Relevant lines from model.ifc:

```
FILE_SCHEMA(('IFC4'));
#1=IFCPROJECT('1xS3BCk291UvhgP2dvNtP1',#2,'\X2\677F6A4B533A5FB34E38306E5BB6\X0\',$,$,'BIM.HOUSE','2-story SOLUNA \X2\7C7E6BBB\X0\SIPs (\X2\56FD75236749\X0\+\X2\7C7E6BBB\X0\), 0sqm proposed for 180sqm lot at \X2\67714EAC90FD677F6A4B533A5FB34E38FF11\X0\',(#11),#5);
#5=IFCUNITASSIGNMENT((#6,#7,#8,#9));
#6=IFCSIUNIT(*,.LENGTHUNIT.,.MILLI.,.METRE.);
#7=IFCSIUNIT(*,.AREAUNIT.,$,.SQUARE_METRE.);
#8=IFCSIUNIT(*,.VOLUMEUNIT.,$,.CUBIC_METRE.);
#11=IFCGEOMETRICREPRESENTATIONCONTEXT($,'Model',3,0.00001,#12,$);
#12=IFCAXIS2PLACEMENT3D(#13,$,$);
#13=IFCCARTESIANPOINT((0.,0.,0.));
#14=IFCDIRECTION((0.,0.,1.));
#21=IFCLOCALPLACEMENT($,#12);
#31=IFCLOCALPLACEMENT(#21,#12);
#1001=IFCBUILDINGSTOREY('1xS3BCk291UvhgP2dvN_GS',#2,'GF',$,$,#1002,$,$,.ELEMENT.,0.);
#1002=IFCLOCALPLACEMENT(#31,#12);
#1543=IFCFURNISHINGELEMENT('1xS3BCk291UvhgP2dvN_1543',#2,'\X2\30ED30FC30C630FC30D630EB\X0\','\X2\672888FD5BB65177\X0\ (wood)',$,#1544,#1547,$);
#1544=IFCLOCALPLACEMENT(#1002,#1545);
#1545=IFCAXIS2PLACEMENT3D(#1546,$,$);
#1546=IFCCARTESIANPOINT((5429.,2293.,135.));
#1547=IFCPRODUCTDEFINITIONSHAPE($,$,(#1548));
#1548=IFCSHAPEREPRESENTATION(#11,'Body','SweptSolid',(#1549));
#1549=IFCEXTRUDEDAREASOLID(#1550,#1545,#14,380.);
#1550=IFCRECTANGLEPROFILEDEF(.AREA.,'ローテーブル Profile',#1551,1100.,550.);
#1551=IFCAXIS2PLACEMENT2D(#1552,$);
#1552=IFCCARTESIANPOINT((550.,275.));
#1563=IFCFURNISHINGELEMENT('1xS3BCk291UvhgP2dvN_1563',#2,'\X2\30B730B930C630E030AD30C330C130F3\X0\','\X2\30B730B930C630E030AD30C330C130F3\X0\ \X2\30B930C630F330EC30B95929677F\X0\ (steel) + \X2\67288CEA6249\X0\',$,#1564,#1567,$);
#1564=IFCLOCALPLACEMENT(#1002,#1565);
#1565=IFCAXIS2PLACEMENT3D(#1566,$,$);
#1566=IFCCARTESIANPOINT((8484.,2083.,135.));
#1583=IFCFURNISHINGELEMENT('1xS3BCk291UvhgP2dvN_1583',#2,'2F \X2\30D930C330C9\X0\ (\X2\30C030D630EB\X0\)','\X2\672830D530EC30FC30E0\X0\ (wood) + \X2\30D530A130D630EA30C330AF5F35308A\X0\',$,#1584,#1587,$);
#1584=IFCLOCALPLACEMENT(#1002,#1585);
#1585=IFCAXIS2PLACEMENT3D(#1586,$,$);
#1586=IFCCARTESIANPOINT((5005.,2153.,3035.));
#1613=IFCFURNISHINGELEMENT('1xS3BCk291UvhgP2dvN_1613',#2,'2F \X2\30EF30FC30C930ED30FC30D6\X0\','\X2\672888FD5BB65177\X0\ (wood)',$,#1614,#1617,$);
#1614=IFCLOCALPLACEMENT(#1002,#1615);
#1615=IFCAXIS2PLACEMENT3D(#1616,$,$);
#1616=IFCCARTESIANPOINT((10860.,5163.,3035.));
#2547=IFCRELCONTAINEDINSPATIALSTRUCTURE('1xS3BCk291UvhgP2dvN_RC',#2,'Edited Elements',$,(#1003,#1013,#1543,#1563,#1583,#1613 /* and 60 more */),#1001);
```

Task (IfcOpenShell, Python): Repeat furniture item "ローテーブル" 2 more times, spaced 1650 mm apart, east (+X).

```python
import numpy as np
import ifcopenshell
import ifcopenshell.api.geometry
import ifcopenshell.api.root
import ifcopenshell.util.element
import ifcopenshell.util.placement
import ifcopenshell.util.unit

model = ifcopenshell.open("model.ifc")
unit_scale = ifcopenshell.util.unit.calculate_unit_scale(model)


def reuse_history(source, copy):
    """copy_class also copies each property set's owner history, people and application; keep the originals."""
    for rel in copy.IsDefinedBy:
        if rel.is_a("IfcRelDefinesByProperties") and (history := rel.RelatingPropertyDefinition.OwnerHistory):
            rel.RelatingPropertyDefinition.OwnerHistory = source.OwnerHistory
            ifcopenshell.util.element.remove_deep2(model, history)


source = model.by_id(1543)
base = ifcopenshell.util.placement.get_local_placement(source.ObjectPlacement)
step = np.array([1.0, 0.0, 0.0]) * 1.65 / unit_scale

for i in range(1, 3):
    copy = ifcopenshell.api.root.copy_class(model, product=source)
    copy.Representation = ifcopenshell.util.element.copy_deep(
        model, source.Representation, exclude=["IfcGeometricRepresentationContext", "IfcRepresentationMap"]
    )
    reuse_history(source, copy)
    matrix = base.copy()
    matrix[:3, 3] += i * step
    print("added at", matrix[:3, 3].round(3) + 0.0)
    ifcopenshell.api.geometry.edit_object_placement(model, product=copy, matrix=matrix, is_si=False)

model.write("model-out.ifc")
```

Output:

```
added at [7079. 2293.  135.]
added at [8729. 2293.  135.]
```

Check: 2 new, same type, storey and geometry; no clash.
